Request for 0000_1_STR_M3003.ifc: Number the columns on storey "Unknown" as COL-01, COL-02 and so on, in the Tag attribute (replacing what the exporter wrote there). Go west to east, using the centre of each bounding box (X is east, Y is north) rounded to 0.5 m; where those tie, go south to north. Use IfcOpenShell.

First a look at what the model holds.

```python
import ifcopenshell
import ifcopenshell.util.element
import ifcopenshell.util.placement

model = ifcopenshell.open("0000_1_STR_M3003.ifc")
print(model.schema)
storey = next(s for s in model.by_type("IfcBuildingStorey") if s.Name == "Unknown")
columns = [e for e in ifcopenshell.util.element.get_decomposition(storey) if e.is_a("IfcColumn")]
for e in sorted(columns, key=lambda e: e.id()):
    origin = ifcopenshell.util.placement.get_local_placement(e.ObjectPlacement)[:3, 3]
    print(e.id(), e.Tag, e.Name, origin.round(2) + 0.0, sep=" | ")
```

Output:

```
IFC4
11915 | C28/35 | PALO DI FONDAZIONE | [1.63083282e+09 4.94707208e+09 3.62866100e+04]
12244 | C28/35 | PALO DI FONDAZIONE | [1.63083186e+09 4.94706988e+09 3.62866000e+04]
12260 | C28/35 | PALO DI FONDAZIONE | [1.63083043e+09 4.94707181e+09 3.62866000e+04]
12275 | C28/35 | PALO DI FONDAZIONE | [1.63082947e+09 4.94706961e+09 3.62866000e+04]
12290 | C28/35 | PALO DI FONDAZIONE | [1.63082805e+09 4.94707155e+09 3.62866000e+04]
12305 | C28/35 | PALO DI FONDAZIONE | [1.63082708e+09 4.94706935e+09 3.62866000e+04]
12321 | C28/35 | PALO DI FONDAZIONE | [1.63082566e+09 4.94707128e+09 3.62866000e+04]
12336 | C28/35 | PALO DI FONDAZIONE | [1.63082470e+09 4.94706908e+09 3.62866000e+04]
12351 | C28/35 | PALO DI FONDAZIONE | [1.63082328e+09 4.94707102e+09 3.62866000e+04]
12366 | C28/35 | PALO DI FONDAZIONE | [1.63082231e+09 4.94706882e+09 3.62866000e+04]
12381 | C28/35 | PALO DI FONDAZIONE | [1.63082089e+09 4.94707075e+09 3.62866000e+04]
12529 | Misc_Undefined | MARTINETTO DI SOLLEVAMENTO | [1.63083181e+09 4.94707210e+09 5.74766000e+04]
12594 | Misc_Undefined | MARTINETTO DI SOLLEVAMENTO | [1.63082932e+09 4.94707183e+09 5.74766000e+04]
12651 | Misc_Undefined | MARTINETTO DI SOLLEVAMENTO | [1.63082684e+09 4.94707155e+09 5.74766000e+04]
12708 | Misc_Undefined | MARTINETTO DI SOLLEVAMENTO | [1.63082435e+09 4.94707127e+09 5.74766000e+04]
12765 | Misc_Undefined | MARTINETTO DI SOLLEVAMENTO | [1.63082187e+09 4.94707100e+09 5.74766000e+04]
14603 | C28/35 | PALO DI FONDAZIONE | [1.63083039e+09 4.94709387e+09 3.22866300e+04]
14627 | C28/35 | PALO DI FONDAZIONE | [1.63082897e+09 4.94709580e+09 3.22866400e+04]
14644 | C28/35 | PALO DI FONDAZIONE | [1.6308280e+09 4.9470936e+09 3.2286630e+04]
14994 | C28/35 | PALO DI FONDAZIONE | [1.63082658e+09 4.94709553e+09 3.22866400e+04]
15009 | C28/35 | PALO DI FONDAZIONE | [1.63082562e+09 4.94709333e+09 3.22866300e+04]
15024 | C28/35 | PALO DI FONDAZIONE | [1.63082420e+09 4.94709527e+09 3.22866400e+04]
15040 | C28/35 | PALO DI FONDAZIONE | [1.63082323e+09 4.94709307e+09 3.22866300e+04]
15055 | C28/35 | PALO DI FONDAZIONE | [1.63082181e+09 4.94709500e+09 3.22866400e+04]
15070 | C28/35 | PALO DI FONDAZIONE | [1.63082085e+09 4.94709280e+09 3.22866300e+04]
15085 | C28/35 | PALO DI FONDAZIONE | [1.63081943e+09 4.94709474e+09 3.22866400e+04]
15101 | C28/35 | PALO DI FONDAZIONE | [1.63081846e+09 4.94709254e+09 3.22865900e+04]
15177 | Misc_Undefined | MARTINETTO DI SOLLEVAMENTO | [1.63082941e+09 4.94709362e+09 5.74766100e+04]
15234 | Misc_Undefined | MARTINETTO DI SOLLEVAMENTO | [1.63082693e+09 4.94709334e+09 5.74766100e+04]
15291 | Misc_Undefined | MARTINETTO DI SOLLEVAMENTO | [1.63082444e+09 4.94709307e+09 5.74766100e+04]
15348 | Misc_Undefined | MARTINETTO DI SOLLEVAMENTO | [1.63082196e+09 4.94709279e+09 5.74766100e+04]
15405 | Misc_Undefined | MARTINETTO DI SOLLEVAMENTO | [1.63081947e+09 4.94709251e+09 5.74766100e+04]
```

```python
import ifcopenshell
import ifcopenshell.geom
import ifcopenshell.util.element
import ifcopenshell.util.shape

model = ifcopenshell.open("0000_1_STR_M3003.ifc")
settings = ifcopenshell.geom.settings()
settings.set("use-world-coords", True)


def centre(element):
    shape = ifcopenshell.geom.create_shape(settings, element)
    return ifcopenshell.util.shape.get_bbox_centroid(shape.geometry)


storey = next(s for s in model.by_type("IfcBuildingStorey") if s.Name == "Unknown")
columns = [e for e in ifcopenshell.util.element.get_decomposition(storey) if e.is_a("IfcColumn")]

# Insertion points can sit at a corner or the storey origin, so sort by the geometry (in metres).
centres = {e: centre(e) for e in columns}
columns.sort(key=lambda e: (round(centres[e][0] / 0.5), centres[e][1]))

for i, e in enumerate(columns, start=1):
    number = f"COL-{i:02d}"
    e.Tag = number
    print(e.id(), number)

model.write("0000_1_STR_M3003_rev.ifc")
```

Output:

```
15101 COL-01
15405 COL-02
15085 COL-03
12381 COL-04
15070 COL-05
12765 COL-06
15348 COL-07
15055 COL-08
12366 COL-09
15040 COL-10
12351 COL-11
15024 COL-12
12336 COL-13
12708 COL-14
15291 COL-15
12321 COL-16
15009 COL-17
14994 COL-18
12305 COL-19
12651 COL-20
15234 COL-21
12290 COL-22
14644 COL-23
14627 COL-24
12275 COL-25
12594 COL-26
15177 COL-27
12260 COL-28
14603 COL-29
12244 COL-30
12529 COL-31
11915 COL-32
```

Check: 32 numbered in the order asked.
